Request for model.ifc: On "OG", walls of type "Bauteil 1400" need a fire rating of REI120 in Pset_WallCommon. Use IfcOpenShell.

First a look at what the model holds.

```python
import ifcopenshell
import ifcopenshell.util.element

model = ifcopenshell.open("model.ifc")
print(model.schema)
storey = next(s for s in model.by_type("IfcBuildingStorey") if s.Name == "OG")
walls = [e for e in ifcopenshell.util.element.get_decomposition(storey) if e.is_a("IfcWall")]
seen = {}
for e in walls:
    element_type = ifcopenshell.util.element.get_type(e)
    key = (element_type.Name if element_type != e and element_type else None, ifcopenshell.util.element.get_pset(e, "Pset_WallCommon", "FireRating"))
    seen[key] = seen.get(key, 0) + 1
for (name, value), count in sorted(seen.items(), key=str):
    print(count, "x", name, "|", value)
```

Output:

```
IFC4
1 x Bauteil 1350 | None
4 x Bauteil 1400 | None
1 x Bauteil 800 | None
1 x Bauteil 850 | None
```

```python
import ifcopenshell
import ifcopenshell.api.pset
import ifcopenshell.util.element

model = ifcopenshell.open("model.ifc")

storey = next(s for s in model.by_type("IfcBuildingStorey") if s.Name == "OG")
walls = [e for e in ifcopenshell.util.element.get_decomposition(storey) if e.is_a("IfcWall")]

count = 0
for e in walls:
    element_type = ifcopenshell.util.element.get_type(e)
    if element_type in (None, e) or element_type.Name != "Bauteil 1400":
        continue
    # add_pset returns the element's existing set when there is one.
    pset = ifcopenshell.api.pset.add_pset(model, product=e, name="Pset_WallCommon")
    ifcopenshell.api.pset.edit_pset(model, pset=pset, properties={"FireRating": "REI120"})
    count += 1

print(count, "walls updated")

model.write("model_rev.ifc")
```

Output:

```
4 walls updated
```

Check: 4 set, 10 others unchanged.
